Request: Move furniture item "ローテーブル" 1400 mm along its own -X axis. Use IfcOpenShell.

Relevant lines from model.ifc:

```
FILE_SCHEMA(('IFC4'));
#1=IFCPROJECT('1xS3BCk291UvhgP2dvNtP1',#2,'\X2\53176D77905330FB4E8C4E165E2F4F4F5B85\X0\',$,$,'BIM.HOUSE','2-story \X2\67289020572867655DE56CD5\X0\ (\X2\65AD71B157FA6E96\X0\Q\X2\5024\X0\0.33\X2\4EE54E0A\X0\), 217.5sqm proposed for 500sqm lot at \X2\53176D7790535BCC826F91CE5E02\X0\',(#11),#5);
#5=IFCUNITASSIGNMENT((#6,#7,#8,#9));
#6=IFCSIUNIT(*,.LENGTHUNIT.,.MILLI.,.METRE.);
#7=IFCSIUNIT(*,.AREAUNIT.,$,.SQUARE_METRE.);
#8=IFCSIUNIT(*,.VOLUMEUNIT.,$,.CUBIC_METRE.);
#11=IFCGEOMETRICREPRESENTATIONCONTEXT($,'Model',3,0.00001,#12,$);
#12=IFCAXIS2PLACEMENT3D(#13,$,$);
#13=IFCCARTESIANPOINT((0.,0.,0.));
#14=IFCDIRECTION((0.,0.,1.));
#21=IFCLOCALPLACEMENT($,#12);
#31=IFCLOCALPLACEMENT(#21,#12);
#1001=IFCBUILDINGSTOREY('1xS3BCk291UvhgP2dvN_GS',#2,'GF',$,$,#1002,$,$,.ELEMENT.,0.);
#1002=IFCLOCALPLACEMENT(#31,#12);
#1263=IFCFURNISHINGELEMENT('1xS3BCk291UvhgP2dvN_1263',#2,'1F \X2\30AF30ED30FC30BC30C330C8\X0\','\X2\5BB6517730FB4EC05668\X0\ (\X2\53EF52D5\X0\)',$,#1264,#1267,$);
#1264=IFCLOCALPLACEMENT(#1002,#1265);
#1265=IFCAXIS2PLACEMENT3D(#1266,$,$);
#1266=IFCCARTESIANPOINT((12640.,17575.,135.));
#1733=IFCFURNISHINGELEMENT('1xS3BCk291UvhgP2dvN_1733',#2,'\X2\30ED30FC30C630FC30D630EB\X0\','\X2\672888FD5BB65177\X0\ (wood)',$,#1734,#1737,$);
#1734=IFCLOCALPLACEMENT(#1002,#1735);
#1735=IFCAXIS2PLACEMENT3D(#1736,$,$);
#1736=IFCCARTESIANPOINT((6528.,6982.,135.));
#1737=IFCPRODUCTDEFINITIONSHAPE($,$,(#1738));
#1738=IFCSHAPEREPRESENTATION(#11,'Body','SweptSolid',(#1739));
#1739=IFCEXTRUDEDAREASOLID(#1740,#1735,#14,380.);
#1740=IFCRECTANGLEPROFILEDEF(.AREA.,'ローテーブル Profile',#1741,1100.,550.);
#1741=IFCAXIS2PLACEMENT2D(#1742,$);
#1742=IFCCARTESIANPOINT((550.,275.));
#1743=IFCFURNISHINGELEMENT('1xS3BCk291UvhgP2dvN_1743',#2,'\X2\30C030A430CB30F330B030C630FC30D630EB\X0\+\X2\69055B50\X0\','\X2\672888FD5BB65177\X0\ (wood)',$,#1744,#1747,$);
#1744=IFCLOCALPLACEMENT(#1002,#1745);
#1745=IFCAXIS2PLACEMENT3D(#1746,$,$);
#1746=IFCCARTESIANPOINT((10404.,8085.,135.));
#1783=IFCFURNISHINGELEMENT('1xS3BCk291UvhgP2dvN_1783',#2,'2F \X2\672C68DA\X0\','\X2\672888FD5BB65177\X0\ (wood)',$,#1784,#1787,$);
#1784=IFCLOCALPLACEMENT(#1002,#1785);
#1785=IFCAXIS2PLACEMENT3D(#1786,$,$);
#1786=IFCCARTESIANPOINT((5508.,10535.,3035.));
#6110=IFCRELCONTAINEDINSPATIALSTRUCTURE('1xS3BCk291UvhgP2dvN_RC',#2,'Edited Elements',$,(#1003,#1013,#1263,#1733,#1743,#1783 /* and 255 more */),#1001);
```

```python
import ifcopenshell
import ifcopenshell.api.geometry
import ifcopenshell.util.placement

model = ifcopenshell.open("model.ifc")

item = model.by_id(1733)
matrix = ifcopenshell.util.placement.get_local_placement(item.ObjectPlacement)
matrix[:3, 3] -= matrix[:3, 0] * 1400.0
ifcopenshell.api.geometry.edit_object_placement(model, product=item, matrix=matrix, is_si=False)

print(ifcopenshell.util.placement.get_local_placement(item.ObjectPlacement).round(3) + 0.0)

model.write("model_edited.ifc")
```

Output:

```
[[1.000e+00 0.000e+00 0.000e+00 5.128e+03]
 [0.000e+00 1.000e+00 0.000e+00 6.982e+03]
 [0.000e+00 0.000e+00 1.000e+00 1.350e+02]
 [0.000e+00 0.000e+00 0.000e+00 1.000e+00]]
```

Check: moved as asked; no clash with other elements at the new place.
